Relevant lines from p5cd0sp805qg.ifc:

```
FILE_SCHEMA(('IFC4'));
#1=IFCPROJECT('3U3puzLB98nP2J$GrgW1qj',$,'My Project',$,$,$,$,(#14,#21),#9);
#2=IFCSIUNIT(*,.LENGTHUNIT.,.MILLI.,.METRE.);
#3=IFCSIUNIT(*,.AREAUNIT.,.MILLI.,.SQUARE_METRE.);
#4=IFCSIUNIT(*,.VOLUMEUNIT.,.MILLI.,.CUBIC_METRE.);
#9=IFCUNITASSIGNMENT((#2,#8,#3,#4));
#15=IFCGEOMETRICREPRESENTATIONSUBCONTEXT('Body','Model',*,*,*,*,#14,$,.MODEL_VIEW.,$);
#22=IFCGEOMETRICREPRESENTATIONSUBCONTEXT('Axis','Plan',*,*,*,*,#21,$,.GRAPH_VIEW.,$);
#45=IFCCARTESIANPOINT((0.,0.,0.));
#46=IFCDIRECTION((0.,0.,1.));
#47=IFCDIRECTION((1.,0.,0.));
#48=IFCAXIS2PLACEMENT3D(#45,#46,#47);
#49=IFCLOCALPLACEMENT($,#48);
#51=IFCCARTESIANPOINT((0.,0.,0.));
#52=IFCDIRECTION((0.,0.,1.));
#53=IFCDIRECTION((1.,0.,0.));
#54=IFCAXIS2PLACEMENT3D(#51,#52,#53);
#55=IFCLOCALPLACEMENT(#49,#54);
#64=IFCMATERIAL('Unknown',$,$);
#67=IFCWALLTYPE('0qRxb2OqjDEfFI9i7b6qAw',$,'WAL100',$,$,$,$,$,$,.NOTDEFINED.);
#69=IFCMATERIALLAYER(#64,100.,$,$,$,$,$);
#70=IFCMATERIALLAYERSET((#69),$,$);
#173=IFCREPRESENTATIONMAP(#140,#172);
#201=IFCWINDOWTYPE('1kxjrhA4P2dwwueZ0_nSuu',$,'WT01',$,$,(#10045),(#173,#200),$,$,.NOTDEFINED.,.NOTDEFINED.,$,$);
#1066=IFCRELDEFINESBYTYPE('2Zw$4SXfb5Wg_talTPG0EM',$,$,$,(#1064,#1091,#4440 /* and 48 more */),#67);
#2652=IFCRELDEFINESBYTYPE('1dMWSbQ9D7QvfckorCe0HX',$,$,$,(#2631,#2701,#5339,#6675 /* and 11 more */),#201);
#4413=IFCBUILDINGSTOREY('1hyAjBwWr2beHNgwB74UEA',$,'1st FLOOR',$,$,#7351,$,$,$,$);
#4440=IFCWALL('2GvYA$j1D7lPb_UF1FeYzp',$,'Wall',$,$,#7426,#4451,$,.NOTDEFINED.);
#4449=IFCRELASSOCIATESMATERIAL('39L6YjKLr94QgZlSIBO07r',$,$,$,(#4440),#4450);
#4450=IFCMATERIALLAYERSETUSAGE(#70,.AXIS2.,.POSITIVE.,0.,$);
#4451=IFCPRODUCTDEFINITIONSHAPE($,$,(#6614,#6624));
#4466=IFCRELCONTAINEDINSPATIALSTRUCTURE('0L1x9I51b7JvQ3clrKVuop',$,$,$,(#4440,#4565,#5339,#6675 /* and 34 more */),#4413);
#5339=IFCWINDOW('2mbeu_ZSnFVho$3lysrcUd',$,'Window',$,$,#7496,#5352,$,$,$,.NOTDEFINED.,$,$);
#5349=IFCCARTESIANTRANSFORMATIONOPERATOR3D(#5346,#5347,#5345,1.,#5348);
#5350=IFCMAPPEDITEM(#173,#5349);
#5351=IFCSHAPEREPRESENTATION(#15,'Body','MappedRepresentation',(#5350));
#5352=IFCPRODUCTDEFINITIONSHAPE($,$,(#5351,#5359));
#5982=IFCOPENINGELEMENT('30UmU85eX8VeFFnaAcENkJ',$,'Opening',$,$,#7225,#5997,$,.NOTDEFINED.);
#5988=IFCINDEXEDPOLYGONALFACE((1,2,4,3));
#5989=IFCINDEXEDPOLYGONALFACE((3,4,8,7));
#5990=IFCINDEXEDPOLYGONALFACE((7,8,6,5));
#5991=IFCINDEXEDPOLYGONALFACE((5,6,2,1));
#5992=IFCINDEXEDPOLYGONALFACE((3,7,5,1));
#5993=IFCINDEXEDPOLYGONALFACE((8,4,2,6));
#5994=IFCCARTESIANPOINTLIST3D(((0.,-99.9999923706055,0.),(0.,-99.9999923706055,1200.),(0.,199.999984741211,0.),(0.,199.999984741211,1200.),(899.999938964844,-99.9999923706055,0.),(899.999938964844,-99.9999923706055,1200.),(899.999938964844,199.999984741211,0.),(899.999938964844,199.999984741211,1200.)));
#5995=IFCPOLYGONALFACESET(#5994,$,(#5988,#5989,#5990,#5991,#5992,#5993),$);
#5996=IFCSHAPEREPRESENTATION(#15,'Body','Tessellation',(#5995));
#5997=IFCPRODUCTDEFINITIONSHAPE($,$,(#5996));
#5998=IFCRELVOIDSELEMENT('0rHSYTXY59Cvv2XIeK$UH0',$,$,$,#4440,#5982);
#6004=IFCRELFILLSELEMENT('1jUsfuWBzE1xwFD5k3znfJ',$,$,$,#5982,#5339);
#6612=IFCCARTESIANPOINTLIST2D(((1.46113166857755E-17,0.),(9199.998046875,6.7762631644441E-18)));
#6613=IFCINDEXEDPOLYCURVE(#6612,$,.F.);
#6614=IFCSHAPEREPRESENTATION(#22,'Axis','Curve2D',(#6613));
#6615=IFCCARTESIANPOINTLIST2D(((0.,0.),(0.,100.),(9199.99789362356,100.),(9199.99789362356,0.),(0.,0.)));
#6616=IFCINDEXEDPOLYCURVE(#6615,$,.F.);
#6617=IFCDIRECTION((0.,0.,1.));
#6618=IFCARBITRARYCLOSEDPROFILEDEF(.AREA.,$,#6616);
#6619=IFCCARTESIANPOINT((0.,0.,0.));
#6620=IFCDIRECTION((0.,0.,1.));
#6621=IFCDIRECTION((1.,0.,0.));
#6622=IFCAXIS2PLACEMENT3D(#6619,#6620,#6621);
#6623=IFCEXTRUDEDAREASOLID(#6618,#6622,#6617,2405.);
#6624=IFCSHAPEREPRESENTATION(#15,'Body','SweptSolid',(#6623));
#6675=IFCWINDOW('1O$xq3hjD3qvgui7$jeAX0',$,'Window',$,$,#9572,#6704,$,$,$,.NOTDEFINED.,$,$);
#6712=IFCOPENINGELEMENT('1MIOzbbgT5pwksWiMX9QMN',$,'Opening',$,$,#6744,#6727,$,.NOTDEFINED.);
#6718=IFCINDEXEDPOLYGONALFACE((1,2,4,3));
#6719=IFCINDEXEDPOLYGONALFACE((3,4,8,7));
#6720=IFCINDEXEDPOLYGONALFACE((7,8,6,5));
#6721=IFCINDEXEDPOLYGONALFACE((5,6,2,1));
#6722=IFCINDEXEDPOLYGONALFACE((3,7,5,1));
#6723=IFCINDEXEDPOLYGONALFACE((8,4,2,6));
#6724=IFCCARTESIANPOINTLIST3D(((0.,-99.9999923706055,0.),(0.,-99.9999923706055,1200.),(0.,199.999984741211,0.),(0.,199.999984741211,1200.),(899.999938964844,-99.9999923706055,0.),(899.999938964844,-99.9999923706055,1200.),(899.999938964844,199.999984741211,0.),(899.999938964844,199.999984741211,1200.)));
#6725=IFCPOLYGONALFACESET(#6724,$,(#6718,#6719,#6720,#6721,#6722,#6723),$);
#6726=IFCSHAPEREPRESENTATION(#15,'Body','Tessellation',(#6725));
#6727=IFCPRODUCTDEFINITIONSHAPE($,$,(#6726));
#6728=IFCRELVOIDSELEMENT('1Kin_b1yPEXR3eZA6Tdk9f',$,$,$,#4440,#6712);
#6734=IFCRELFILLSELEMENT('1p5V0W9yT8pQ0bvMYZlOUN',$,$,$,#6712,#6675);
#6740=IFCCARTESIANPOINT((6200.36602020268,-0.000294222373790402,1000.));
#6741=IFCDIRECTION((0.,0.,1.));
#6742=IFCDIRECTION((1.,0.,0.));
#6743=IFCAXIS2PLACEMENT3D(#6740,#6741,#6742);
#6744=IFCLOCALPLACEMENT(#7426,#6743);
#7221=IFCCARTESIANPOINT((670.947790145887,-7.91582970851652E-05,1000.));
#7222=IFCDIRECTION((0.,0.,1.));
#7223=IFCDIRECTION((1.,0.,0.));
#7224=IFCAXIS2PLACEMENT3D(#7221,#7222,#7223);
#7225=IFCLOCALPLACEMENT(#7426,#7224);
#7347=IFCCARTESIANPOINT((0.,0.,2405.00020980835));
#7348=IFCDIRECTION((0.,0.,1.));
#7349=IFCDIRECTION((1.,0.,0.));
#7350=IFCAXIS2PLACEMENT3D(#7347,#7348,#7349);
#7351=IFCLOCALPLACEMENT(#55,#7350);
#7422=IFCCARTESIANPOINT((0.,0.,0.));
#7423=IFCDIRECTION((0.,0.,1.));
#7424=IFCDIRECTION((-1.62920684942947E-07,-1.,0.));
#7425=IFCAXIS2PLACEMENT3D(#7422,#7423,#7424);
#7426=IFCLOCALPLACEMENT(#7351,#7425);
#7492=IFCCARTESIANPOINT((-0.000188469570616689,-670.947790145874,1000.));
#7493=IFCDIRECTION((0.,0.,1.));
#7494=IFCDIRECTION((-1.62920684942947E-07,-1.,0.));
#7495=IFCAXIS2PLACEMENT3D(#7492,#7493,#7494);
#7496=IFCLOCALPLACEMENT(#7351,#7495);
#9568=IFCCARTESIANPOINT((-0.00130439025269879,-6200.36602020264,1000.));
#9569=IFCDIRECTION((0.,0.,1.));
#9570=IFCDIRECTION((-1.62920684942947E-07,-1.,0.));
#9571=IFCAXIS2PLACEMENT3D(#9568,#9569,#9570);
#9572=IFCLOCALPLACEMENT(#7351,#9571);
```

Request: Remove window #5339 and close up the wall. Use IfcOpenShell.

```python
import ifcopenshell
import ifcopenshell.api.feature
import ifcopenshell.api.root
import ifcopenshell.geom
import ifcopenshell.util.shape

model = ifcopenshell.open("p5cd0sp805qg.ifc")
settings = ifcopenshell.geom.settings()


def volume(element):
    """Net volume in cubic metres, openings subtracted."""
    shape = ifcopenshell.geom.create_shape(settings, element)
    return ifcopenshell.util.shape.get_volume(shape.geometry)


window = model.by_guid("2mbeu_ZSnFVho$3lysrcUd")
opening = window.FillsVoids[0].RelatingOpeningElement
wall = opening.VoidsElements[0].RelatingBuildingElement
before = volume(wall)

ifcopenshell.api.root.remove_product(model, product=window)
ifcopenshell.api.feature.remove_feature(model, feature=opening)

after = volume(wall)

print(f"wall volume {before:.3f} -> {after:.3f} m3")

model.write("p5cd0sp805qg_edited.ifc")
```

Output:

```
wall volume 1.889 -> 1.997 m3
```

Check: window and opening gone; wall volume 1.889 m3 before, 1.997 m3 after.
